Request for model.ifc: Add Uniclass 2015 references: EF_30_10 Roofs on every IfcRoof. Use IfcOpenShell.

First a look at what the model holds.

```python
import ifcopenshell

model = ifcopenshell.open("model.ifc")
print(model.schema)
print("classifications:", [c.Name for c in model.by_type("IfcClassification")])
for ifc_class in ("IfcDoor", "IfcRoof", "IfcStair", "IfcWall", "IfcWindow"):
    print(ifc_class, len(model.by_type(ifc_class)))
```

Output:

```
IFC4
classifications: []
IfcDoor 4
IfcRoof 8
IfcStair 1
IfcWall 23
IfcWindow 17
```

```python
import ifcopenshell
import ifcopenshell.api.classification

model = ifcopenshell.open("model.ifc")

system = ifcopenshell.api.classification.add_classification(model, classification="Uniclass 2015")

codes = {
    "IfcRoof": ("EF_30_10", "Roofs"),
}
for ifc_class, (code, name) in codes.items():
    products = model.by_type(ifc_class)
    ifcopenshell.api.classification.add_reference(
        model, products=products, classification=system, identification=code, name=name
    )
    print(code, len(products))

model.write("model_edited.ifc")
```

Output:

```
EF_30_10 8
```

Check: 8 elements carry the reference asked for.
